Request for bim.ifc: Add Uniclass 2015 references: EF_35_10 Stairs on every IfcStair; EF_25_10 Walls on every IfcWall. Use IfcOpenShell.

First a look at what the model holds.

```python
import ifcopenshell

model = ifcopenshell.open("bim.ifc")
print(model.schema)
print("classifications:", [c.Name for c in model.by_type("IfcClassification")])
for ifc_class in ("IfcDoor", "IfcRoof", "IfcStair", "IfcWall", "IfcWindow"):
    print(ifc_class, len(model.by_type(ifc_class)))
```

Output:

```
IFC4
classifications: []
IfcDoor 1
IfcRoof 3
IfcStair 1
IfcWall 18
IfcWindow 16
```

```python
import ifcopenshell
import ifcopenshell.api.classification

model = ifcopenshell.open("bim.ifc")

system = ifcopenshell.api.classification.add_classification(model, classification="Uniclass 2015")

codes = {
    "IfcStair": ("EF_35_10", "Stairs"),
    "IfcWall": ("EF_25_10", "Walls"),
}
for ifc_class, (code, name) in codes.items():
    products = model.by_type(ifc_class)
    ifcopenshell.api.classification.add_reference(
        model, products=products, classification=system, identification=code, name=name
    )
    print(code, len(products))

model.write("bim_updated.ifc")
```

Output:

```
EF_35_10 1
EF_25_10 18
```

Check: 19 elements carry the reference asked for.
